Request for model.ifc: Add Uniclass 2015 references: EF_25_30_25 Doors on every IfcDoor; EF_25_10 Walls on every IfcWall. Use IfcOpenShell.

First a look at what the model holds.

```python
import ifcopenshell

model = ifcopenshell.open("model.ifc")
print(model.schema)
print("classifications:", [c.Name for c in model.by_type("IfcClassification")])
for ifc_class in ("IfcDoor", "IfcRoof", "IfcStair", "IfcWall", "IfcWindow"):
    print(ifc_class, len(model.by_type(ifc_class)))
```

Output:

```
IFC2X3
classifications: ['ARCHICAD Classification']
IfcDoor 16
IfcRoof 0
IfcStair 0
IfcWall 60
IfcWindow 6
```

```python
import ifcopenshell
import ifcopenshell.api.classification

model = ifcopenshell.open("model.ifc")

# IFC2X3 requires Source and Edition and has no link from the project to the system.
system = model.create_entity("IfcClassification", Source="NBS", Edition="2015", Name="Uniclass 2015")

codes = {
    "IfcDoor": ("EF_25_30_25", "Doors"),
    "IfcWall": ("EF_25_10", "Walls"),
}
for ifc_class, (code, name) in codes.items():
    products = model.by_type(ifc_class)
    ifcopenshell.api.classification.add_reference(
        model, products=products, classification=system, identification=code, name=name
    )
    print(code, len(products))

model.write("model_edited.ifc")
```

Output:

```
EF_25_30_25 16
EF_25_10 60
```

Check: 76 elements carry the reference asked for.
